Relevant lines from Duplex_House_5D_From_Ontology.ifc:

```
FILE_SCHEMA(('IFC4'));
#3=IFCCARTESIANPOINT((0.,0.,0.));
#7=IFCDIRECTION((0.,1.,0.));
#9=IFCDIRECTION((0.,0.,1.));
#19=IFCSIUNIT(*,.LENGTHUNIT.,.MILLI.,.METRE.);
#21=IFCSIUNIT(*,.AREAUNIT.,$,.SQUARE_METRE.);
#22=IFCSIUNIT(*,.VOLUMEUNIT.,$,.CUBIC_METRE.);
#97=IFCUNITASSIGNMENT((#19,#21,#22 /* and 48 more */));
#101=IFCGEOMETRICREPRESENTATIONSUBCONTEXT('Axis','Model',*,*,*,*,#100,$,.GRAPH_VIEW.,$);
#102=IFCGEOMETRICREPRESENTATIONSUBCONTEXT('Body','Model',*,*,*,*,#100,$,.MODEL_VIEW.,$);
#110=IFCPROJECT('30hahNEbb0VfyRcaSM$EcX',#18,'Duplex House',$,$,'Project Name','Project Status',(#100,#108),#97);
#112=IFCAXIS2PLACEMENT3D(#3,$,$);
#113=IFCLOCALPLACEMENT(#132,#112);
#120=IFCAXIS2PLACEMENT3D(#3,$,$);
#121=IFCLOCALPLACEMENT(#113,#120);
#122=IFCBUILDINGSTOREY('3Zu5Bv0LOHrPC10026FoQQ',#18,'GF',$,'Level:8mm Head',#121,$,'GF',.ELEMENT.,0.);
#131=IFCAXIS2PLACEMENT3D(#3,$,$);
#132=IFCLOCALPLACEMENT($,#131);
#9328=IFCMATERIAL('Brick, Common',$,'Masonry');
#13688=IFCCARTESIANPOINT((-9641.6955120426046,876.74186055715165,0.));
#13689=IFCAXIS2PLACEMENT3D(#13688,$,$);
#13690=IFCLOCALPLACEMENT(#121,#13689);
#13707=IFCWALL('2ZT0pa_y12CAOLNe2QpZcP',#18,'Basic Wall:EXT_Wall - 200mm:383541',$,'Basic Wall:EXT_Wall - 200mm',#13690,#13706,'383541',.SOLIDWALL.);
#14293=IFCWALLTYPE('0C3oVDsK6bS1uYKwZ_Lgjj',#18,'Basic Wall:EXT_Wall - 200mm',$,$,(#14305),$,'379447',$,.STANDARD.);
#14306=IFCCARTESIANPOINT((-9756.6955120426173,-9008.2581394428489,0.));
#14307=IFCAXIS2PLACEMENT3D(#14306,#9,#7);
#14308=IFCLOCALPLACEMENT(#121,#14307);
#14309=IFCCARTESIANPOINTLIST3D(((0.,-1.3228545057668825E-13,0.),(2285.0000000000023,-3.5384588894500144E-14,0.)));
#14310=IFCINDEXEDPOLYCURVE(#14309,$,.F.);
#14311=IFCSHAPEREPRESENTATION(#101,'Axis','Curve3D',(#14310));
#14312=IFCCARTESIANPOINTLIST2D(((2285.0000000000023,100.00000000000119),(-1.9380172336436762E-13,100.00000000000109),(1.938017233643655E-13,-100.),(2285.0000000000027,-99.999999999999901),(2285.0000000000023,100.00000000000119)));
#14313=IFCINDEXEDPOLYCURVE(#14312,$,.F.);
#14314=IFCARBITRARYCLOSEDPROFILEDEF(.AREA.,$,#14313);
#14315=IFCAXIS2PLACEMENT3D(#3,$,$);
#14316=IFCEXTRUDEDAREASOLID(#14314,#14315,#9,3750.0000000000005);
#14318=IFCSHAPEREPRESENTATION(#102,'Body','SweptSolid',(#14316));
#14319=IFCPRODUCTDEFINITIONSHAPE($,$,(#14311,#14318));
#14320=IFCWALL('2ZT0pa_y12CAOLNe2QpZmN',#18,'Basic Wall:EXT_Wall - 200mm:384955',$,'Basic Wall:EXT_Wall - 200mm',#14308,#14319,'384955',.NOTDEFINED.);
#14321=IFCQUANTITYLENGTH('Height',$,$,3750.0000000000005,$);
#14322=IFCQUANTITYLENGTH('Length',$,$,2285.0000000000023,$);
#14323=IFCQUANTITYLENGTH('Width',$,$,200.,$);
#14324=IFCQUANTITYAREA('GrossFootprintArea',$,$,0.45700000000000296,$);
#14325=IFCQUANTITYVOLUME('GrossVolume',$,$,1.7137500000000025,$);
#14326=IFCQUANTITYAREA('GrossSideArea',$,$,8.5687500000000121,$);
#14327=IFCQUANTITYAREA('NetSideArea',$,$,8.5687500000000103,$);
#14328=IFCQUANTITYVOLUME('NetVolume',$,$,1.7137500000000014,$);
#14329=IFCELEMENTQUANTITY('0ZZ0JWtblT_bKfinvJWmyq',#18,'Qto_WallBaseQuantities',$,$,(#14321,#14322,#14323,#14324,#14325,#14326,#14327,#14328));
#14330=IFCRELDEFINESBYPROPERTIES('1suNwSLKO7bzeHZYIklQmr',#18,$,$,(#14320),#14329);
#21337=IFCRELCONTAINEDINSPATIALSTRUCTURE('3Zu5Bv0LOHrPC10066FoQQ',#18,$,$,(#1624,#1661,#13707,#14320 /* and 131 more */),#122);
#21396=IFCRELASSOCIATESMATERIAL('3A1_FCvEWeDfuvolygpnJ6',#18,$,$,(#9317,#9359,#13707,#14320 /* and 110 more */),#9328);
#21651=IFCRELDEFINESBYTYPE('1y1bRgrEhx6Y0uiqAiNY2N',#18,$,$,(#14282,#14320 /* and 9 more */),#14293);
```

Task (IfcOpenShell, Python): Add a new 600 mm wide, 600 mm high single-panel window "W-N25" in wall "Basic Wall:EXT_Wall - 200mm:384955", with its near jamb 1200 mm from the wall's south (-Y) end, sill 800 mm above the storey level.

```python
import numpy as np
import ifcopenshell
import ifcopenshell.api.feature
import ifcopenshell.api.geometry
import ifcopenshell.api.pset
import ifcopenshell.api.root
import ifcopenshell.api.spatial
import ifcopenshell.geom
import ifcopenshell.util.element
import ifcopenshell.util.placement
import ifcopenshell.util.representation
import ifcopenshell.util.shape
import ifcopenshell.util.unit

model = ifcopenshell.open("Duplex_House_5D_From_Ontology.ifc")
unit_scale = ifcopenshell.util.unit.calculate_unit_scale(model)
area_scale = ifcopenshell.util.unit.calculate_unit_scale(model, "AREAUNIT")
volume_scale = ifcopenshell.util.unit.calculate_unit_scale(model, "VOLUMEUNIT")
settings = ifcopenshell.geom.settings()


def volume(element):
    """Net volume in cubic metres, openings subtracted."""
    shape = ifcopenshell.geom.create_shape(settings, element)
    return ifcopenshell.util.shape.get_volume(shape.geometry)


wall = model.by_id(14320)
storey = ifcopenshell.util.element.get_container(wall, ifc_class="IfcBuildingStorey")
context = ifcopenshell.util.representation.get_context(model, "Model", "Body", "MODEL_VIEW")
before = volume(wall)

width, height, from_end, sill = 0.6, 0.6, 1.2, 0.8  # metres

# The wall runs along its own X axis, and the end named is its -X end.
wall_shape = ifcopenshell.geom.create_shape(settings, wall)
x, y, z = ifcopenshell.util.shape.get_vertices(wall_shape.geometry).T
start = x.min() + from_end
face, thickness = float(y.min()), float(y.max() - y.min())
wall_matrix = ifcopenshell.util.placement.get_local_placement(wall.ObjectPlacement)
level = ifcopenshell.util.placement.get_local_placement(storey.ObjectPlacement)[2, 3]


def in_wall(x, y):
    """Placement at x, y metres in the wall's axes, at sill height."""
    matrix = wall_matrix.copy()
    matrix[:, 3] = wall_matrix @ np.array([x / unit_scale, y / unit_scale, 0.0, 1.0])
    matrix[2, 3] = level + sill / unit_scale
    return matrix


# Opening: a box that overshoots both wall faces by 50 mm.
opening = ifcopenshell.api.root.create_entity(model, ifc_class="IfcOpeningElement", predefined_type="OPENING")
box = ifcopenshell.api.geometry.add_wall_representation(
    model, context=context, length=width, height=height, thickness=thickness + 0.1
)
ifcopenshell.api.geometry.assign_representation(model, product=opening, representation=box)
ifcopenshell.api.geometry.edit_object_placement(model, product=opening, matrix=in_wall(start, face - 0.05), is_si=False)
ifcopenshell.api.feature.add_feature(model, feature=opening, element=wall)

window = ifcopenshell.api.root.create_entity(model, ifc_class="IfcWindow", name="W-N25", predefined_type="WINDOW")
window.OverallWidth, window.OverallHeight = width / unit_scale, height / unit_scale
window.PartitioningType = "SINGLE_PANEL"
body = ifcopenshell.api.geometry.add_window_representation(
    model,
    context=context,
    overall_width=window.OverallWidth,
    overall_height=window.OverallHeight,
    partition_type="SINGLE_PANEL",
)
ifcopenshell.api.geometry.assign_representation(model, product=window, representation=body)
ifcopenshell.api.spatial.assign_container(model, products=[window], relating_structure=storey)
ifcopenshell.api.feature.add_filling(model, opening=opening, element=window)

# Centre the window in the wall's thickness.
ifcopenshell.api.geometry.edit_object_placement(model, product=window, matrix=in_wall(start, face), is_si=False)
window_shape = ifcopenshell.geom.create_shape(settings, window)
depth = ifcopenshell.util.shape.get_vertices(window_shape.geometry)[:, 1]
offset = face + thickness / 2 - (depth.min() + depth.max()) / 2
ifcopenshell.api.geometry.edit_object_placement(model, product=window, matrix=in_wall(start, offset), is_si=False)

after = volume(wall)

# Update the wall's stored quantities.
qto = model.by_id(ifcopenshell.util.element.get_pset(wall, "Qto_WallBaseQuantities", should_inherit=False)["id"])
ifcopenshell.api.pset.edit_qto(model, qto=qto, properties={
    "NetSideArea": after / thickness / area_scale,
    "NetVolume": after / volume_scale,
})

print(f"wall volume {before:.3f} -> {after:.3f} m3")

model.write("Duplex_House_5D_From_Ontology-out.ifc")
```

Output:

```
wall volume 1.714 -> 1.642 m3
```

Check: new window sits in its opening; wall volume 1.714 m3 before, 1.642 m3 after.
